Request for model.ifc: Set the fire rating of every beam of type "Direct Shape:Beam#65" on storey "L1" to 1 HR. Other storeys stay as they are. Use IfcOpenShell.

First a look at what the model holds.

```python
import ifcopenshell
import ifcopenshell.util.element

model = ifcopenshell.open("model.ifc")
print(model.schema)
storey = next(s for s in model.by_type("IfcBuildingStorey") if s.Name == "L1")
beams = [e for e in ifcopenshell.util.element.get_decomposition(storey) if e.is_a("IfcBeam")]
seen = {}
for e in beams:
    element_type = ifcopenshell.util.element.get_type(e)
    key = (element_type.Name if element_type != e and element_type else None, ifcopenshell.util.element.get_pset(e, "Pset_BeamCommon", "FireRating"))
    seen[key] = seen.get(key, 0) + 1
for (name, value), count in sorted(seen.items(), key=str):
    print(count, "x", name, "|", value)
```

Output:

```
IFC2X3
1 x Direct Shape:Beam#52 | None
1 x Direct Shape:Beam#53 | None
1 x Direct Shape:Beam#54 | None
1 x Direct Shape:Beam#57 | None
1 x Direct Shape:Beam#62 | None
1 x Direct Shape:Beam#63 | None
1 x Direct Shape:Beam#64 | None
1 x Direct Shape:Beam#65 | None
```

```python
import ifcopenshell
import ifcopenshell.api.pset
import ifcopenshell.util.element

model = ifcopenshell.open("model.ifc")

storey = next(s for s in model.by_type("IfcBuildingStorey") if s.Name == "L1")
beams = [e for e in ifcopenshell.util.element.get_decomposition(storey) if e.is_a("IfcBeam")]

count = 0
for e in beams:
    element_type = ifcopenshell.util.element.get_type(e)
    if element_type in (None, e) or element_type.Name != "Direct Shape:Beam#65":
        continue
    # add_pset returns the element's existing set when there is one.
    pset = ifcopenshell.api.pset.add_pset(model, product=e, name="Pset_BeamCommon")
    ifcopenshell.api.pset.edit_pset(model, pset=pset, properties={"FireRating": "1 HR"})
    count += 1

print(count, "beams updated")

model.write("model_updated.ifc")
```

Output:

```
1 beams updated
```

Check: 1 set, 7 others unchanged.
